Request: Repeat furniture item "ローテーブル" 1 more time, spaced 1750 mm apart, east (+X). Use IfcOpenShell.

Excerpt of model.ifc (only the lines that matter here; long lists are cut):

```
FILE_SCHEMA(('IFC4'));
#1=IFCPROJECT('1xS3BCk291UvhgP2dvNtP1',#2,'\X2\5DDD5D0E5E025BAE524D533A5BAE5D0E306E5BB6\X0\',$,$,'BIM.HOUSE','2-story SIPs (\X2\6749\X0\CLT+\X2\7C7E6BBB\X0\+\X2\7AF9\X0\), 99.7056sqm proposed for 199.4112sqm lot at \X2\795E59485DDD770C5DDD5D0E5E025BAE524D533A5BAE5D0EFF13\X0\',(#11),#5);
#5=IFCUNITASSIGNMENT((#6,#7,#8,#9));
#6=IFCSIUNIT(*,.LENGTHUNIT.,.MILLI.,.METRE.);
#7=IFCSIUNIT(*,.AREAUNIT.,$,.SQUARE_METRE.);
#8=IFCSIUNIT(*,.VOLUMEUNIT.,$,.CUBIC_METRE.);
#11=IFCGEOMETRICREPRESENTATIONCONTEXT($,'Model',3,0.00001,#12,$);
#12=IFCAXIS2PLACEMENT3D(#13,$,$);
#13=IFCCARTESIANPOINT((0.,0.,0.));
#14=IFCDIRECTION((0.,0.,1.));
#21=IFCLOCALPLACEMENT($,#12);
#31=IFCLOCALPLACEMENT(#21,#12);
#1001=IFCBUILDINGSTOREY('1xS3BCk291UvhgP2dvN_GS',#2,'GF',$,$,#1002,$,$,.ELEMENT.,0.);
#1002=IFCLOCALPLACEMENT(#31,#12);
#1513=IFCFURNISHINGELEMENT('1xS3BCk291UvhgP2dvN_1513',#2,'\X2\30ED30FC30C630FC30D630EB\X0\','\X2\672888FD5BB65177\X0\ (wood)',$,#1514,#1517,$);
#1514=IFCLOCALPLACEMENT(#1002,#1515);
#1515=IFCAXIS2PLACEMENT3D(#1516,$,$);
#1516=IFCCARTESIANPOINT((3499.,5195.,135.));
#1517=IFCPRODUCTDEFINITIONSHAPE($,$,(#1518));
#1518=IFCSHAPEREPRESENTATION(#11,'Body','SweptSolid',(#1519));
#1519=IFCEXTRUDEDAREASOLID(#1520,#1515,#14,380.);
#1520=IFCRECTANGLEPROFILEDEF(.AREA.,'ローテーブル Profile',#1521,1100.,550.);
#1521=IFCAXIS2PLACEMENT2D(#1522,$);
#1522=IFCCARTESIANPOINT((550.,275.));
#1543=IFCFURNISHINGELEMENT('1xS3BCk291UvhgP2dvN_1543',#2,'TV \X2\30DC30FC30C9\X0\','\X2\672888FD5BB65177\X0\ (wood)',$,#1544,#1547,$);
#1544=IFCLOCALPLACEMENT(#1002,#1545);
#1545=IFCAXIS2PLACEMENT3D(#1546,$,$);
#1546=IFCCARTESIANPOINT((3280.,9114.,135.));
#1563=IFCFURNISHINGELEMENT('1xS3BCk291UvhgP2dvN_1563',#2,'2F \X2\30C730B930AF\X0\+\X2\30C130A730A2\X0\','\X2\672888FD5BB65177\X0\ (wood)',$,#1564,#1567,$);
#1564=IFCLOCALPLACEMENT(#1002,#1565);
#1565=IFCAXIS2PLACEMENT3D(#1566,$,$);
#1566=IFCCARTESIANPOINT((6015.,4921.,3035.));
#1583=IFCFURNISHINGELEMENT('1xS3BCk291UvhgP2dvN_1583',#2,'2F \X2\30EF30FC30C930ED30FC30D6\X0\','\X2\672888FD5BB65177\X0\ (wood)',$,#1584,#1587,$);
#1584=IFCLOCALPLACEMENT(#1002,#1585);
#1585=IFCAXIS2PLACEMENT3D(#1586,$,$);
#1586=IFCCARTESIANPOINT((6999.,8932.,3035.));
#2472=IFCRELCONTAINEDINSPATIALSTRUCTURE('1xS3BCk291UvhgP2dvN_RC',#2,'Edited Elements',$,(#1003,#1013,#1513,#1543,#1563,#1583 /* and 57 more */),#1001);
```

```python
import numpy as np
import ifcopenshell
import ifcopenshell.api.geometry
import ifcopenshell.api.root
import ifcopenshell.util.element
import ifcopenshell.util.placement

model = ifcopenshell.open("model.ifc")


def reuse_history(source, copy):
    """copy_class also copies each property set's owner history, people and application; keep the originals."""
    for rel in copy.IsDefinedBy:
        if rel.is_a("IfcRelDefinesByProperties") and (history := rel.RelatingPropertyDefinition.OwnerHistory):
            rel.RelatingPropertyDefinition.OwnerHistory = source.OwnerHistory
            ifcopenshell.util.element.remove_deep2(model, history)


source = model.by_id(1513)
base = ifcopenshell.util.placement.get_local_placement(source.ObjectPlacement)
step = np.array([1.0, 0.0, 0.0]) * 1750.0

for i in range(1, 2):
    copy = ifcopenshell.api.root.copy_class(model, product=source)
    copy.Representation = ifcopenshell.util.element.copy_deep(
        model, source.Representation, exclude=["IfcGeometricRepresentationContext", "IfcRepresentationMap"]
    )
    reuse_history(source, copy)
    matrix = base.copy()
    matrix[:3, 3] += i * step
    print("added at", matrix[:3, 3].round(3) + 0.0)
    ifcopenshell.api.geometry.edit_object_placement(model, product=copy, matrix=matrix, is_si=False)

model.write("model_rev.ifc")
```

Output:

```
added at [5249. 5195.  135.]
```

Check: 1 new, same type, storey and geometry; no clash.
